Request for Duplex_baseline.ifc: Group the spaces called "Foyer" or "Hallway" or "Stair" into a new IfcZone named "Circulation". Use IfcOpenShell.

First a look at what the model holds.

```python
import ifcopenshell

model = ifcopenshell.open("Duplex_baseline.ifc")
print(model.schema)
seen = {}
for space in model.by_type("IfcSpace"):
    seen[space.LongName] = seen.get(space.LongName, 0) + 1
for name, count in sorted(seen.items(), key=str):
    print(count, "x", name)
print("zones:", [z.Name for z in model.by_type("IfcZone")][:20])
```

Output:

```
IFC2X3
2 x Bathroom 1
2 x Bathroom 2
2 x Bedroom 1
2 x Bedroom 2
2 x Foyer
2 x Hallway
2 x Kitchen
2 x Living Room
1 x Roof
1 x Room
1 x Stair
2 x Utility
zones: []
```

```python
import ifcopenshell
import ifcopenshell.api.group
import ifcopenshell.api.root

model = ifcopenshell.open("Duplex_baseline.ifc")

names = {"Foyer", "Hallway", "Stair"}
spaces = [s for s in model.by_type("IfcSpace") if s.LongName in names]

zone = ifcopenshell.api.root.create_entity(model, ifc_class="IfcZone", name="Circulation")
ifcopenshell.api.group.assign_group(model, products=spaces, group=zone)
print(len(spaces), "spaces in", zone.Name)

model.write("Duplex_baseline-out.ifc")
```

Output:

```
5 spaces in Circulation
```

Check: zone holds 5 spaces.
